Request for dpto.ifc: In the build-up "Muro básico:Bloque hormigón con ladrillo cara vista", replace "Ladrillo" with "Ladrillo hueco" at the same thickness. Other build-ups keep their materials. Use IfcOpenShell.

First a look at what the model holds.

```python
import ifcopenshell
import ifcopenshell.util.element

model = ifcopenshell.open("dpto.ifc")
print(model.schema)
for layer_set in model.by_type("IfcMaterialLayerSet"):
    if layer_set.LayerSetName == "Muro básico:Bloque hormigón con ladrillo cara vista":
        for layer in layer_set.MaterialLayers:
            print(layer.id(), layer.Material and layer.Material.Name, layer.LayerThickness, sep=" | ")
        print(len(ifcopenshell.util.element.get_elements_by_material(model, layer_set)), "elements and types use it")
print(sorted(m.Name for m in model.by_type("IfcMaterial") if m.Name)[:60])
```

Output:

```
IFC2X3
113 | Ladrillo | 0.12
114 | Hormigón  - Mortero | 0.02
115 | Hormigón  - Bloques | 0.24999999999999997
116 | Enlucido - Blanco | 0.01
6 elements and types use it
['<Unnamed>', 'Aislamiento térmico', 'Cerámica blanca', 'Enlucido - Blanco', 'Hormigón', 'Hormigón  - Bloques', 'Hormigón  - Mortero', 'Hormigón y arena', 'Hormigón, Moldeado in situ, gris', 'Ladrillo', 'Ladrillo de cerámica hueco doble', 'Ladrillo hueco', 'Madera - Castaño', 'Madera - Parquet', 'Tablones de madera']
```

```python
import ifcopenshell
import ifcopenshell.api.material

model = ifcopenshell.open("dpto.ifc")

layer_set = next(s for s in model.by_type("IfcMaterialLayerSet") if s.LayerSetName == "Muro básico:Bloque hormigón con ladrillo cara vista")
layer = next(l for l in layer_set.MaterialLayers if l.Material and l.Material.Name == "Ladrillo")
material = next(m for m in model.by_type("IfcMaterial") if m.Name == "Ladrillo hueco")

# Point this one layer at the other material; renaming the old one would change it everywhere.
ifcopenshell.api.material.edit_layer(model, layer=layer, attributes={}, material=material)

print([l.Material.Name if l.Material else None for l in layer_set.MaterialLayers])

model.write("dpto_updated.ifc")
```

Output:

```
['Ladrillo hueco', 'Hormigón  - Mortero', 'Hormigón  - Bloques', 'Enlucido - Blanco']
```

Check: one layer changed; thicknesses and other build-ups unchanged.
